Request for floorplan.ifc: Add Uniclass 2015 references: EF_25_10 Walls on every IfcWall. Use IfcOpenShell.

First a look at what the model holds.

```python
import ifcopenshell

model = ifcopenshell.open("floorplan.ifc")
print(model.schema)
print("classifications:", [c.Name for c in model.by_type("IfcClassification")])
for ifc_class in ("IfcDoor", "IfcRoof", "IfcStair", "IfcWall", "IfcWindow"):
    print(ifc_class, len(model.by_type(ifc_class)))
```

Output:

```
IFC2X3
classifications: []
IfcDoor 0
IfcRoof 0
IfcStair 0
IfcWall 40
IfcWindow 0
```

```python
import ifcopenshell
import ifcopenshell.api.classification

model = ifcopenshell.open("floorplan.ifc")

# IFC2X3 requires Source and Edition and has no link from the project to the system.
system = model.create_entity("IfcClassification", Source="NBS", Edition="2015", Name="Uniclass 2015")

codes = {
    "IfcWall": ("EF_25_10", "Walls"),
}
for ifc_class, (code, name) in codes.items():
    products = model.by_type(ifc_class)
    ifcopenshell.api.classification.add_reference(
        model, products=products, classification=system, identification=code, name=name
    )
    print(code, len(products))

model.write("floorplan_updated.ifc")
```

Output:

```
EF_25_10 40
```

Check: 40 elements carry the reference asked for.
